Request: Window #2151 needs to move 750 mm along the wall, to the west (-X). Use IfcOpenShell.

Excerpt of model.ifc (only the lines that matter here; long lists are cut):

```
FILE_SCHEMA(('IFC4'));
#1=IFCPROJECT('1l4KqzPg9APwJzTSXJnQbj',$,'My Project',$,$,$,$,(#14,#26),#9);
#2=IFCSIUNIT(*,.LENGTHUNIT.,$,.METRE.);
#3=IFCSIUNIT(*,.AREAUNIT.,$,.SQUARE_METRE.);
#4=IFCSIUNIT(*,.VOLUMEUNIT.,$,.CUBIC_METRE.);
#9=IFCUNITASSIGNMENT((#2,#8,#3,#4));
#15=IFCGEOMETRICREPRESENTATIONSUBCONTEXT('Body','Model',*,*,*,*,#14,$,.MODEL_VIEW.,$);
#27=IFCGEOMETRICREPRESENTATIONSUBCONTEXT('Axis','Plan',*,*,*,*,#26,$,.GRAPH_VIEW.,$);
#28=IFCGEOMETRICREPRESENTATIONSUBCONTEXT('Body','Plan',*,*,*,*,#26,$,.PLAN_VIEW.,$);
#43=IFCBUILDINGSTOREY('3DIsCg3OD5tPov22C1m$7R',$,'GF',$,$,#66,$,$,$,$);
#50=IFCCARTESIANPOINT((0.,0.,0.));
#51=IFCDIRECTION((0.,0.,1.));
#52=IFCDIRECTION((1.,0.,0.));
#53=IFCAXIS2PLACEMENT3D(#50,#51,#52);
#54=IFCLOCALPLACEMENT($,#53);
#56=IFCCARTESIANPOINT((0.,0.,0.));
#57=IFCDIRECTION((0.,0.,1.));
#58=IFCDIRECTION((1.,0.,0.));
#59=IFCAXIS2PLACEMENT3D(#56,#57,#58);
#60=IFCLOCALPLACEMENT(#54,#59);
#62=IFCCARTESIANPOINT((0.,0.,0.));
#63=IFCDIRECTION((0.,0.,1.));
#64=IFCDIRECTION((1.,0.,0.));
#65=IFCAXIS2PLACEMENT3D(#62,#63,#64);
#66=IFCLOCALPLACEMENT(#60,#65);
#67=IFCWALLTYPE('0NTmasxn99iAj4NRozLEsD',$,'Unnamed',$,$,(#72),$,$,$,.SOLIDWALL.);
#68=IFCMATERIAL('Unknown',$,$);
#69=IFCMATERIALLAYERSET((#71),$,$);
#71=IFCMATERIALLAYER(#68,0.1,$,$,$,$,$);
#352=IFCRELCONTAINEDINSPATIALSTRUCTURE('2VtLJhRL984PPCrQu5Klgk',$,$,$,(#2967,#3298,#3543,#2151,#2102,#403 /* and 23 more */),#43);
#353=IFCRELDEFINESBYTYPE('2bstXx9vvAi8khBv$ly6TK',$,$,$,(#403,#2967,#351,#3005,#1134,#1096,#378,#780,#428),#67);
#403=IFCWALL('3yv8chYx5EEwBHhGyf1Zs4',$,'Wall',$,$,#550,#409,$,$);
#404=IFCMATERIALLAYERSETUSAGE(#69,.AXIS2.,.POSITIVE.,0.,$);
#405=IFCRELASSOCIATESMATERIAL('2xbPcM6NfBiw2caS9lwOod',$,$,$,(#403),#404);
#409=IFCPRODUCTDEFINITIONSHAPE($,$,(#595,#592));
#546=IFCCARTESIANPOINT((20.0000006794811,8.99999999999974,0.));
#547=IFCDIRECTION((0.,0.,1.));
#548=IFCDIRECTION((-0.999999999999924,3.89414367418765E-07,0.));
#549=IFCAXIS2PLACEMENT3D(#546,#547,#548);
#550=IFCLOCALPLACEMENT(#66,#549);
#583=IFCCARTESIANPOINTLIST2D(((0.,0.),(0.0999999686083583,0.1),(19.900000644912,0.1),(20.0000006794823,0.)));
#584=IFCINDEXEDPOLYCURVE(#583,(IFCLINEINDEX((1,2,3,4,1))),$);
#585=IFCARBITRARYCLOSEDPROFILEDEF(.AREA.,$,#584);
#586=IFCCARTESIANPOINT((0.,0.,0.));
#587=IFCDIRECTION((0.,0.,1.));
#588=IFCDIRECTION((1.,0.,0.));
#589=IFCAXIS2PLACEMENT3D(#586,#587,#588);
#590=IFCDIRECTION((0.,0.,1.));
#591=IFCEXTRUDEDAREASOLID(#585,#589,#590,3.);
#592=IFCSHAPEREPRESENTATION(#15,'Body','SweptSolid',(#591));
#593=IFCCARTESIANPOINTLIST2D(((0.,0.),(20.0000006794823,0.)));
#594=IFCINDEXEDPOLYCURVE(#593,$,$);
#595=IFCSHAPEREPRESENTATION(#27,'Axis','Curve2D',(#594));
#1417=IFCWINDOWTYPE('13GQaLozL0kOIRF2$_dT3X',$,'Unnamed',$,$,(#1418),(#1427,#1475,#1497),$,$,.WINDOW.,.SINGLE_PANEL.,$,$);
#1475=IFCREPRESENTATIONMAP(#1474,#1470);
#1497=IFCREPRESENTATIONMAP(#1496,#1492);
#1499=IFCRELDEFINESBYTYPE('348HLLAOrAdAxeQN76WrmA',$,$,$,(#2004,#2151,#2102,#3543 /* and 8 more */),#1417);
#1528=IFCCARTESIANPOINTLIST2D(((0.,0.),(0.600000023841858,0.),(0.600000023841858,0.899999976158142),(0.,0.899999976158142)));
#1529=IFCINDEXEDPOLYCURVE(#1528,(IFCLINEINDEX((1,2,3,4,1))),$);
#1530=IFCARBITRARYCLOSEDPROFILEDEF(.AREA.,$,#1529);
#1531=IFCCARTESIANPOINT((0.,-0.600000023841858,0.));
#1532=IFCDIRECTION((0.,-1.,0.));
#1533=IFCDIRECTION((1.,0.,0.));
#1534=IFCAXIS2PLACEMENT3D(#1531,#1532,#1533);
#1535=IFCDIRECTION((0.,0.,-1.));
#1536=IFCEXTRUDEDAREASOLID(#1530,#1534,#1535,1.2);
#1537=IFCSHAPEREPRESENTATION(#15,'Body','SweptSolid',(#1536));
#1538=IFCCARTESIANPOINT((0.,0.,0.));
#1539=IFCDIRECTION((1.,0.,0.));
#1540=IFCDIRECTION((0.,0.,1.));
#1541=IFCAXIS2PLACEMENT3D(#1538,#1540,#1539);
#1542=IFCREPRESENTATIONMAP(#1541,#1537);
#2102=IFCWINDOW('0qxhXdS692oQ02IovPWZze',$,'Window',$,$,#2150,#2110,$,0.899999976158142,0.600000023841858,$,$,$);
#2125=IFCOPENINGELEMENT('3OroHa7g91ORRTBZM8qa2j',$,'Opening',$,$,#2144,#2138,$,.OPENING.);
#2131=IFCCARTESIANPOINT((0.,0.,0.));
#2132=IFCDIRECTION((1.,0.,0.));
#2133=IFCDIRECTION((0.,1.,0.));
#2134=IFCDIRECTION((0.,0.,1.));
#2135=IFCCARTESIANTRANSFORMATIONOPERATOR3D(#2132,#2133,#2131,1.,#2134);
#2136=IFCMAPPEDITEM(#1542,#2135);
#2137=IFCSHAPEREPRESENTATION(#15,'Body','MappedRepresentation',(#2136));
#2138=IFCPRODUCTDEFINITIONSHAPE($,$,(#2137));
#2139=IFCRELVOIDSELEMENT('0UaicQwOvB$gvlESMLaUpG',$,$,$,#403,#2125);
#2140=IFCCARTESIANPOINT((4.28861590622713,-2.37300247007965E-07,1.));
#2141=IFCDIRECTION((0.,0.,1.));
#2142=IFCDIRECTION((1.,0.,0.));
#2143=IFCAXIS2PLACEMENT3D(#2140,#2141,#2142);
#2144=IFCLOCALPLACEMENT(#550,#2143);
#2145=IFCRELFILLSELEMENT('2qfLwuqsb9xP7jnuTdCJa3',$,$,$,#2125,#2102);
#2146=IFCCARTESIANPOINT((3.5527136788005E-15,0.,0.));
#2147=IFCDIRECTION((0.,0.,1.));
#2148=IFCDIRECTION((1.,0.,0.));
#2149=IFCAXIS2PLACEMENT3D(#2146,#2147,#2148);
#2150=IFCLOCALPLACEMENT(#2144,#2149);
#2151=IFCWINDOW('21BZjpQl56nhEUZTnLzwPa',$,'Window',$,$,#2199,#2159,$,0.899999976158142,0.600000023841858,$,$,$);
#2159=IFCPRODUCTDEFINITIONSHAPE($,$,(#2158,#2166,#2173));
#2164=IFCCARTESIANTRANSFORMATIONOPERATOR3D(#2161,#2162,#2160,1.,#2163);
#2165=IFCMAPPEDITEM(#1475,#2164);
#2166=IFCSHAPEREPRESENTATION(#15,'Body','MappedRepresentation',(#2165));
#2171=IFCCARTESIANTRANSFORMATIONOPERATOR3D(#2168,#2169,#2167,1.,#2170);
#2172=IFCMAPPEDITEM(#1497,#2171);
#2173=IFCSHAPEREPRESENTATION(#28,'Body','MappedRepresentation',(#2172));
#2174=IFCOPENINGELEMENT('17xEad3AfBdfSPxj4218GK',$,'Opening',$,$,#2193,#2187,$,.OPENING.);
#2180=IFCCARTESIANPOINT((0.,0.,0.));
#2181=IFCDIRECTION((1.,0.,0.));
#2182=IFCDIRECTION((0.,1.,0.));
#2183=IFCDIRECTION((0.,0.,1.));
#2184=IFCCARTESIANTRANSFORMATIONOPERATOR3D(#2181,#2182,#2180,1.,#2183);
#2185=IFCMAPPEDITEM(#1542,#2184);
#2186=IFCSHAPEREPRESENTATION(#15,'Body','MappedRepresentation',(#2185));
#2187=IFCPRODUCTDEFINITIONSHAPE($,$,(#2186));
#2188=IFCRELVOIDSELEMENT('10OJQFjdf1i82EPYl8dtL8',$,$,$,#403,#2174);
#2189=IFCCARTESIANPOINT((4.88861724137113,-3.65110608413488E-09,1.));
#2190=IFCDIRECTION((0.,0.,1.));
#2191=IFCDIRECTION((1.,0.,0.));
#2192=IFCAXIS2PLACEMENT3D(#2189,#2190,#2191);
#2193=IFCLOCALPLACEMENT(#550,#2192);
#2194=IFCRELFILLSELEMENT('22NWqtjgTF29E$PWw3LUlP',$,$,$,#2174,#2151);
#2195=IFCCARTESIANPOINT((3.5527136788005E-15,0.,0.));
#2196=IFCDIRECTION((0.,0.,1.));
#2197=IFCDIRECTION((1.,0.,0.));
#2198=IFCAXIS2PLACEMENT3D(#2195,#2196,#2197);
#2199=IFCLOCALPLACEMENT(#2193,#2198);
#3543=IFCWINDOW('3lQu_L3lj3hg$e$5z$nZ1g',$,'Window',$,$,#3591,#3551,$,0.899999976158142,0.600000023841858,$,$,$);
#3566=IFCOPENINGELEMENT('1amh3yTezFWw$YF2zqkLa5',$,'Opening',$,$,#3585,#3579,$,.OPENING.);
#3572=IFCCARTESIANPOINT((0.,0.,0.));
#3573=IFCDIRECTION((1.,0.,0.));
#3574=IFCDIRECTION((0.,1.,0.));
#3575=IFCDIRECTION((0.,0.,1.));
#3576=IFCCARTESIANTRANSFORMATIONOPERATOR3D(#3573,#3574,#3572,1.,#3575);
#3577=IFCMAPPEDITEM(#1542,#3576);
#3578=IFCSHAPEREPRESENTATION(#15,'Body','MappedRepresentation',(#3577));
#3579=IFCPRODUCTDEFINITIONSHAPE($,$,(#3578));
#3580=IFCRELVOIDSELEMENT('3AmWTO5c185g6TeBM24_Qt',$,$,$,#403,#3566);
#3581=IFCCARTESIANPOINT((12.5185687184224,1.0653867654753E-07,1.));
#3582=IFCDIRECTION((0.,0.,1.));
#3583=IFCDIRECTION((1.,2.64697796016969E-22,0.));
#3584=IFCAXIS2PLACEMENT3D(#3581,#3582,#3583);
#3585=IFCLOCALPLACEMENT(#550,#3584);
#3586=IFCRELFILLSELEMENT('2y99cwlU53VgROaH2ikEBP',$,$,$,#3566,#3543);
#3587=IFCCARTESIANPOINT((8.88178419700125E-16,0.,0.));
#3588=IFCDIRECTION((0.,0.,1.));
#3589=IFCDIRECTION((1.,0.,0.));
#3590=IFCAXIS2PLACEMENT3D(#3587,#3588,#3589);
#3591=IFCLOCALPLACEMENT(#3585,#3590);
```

```python
import ifcopenshell
import ifcopenshell.api.geometry
import ifcopenshell.util.placement
import ifcopenshell.util.unit

model = ifcopenshell.open("model.ifc")
unit_scale = ifcopenshell.util.unit.calculate_unit_scale(model)

window = model.by_guid("21BZjpQl56nhEUZTnLzwPa")
opening = window.FillsVoids[0].RelatingOpeningElement
wall = opening.VoidsElements[0].RelatingBuildingElement

wall_matrix = ifcopenshell.util.placement.get_local_placement(wall.ObjectPlacement)
shift = wall_matrix[:3, 0] * 0.75 / unit_scale
before = ifcopenshell.util.placement.get_local_placement(window.ObjectPlacement)[:3, 3].copy()

# The window is placed relative to its opening, so it follows when the opening moves.
matrix = ifcopenshell.util.placement.get_local_placement(opening.ObjectPlacement)
matrix[:3, 3] += shift
ifcopenshell.api.geometry.edit_object_placement(
    model, product=opening, matrix=matrix, is_si=False, should_transform_children=True
)

after = ifcopenshell.util.placement.get_local_placement(window.ObjectPlacement)[:3, 3]
print("window moved by", (after - before).round(3) + 0.0)

model.write("model_updated.ifc")
```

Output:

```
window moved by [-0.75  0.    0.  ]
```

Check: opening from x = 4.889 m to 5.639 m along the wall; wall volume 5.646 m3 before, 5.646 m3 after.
